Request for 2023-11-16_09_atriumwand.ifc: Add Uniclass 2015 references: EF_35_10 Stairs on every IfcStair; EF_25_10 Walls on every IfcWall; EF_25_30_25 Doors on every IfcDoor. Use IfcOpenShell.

First a look at what the model holds.

```python
import ifcopenshell

model = ifcopenshell.open("2023-11-16_09_atriumwand.ifc")
print(model.schema)
print("classifications:", [c.Name for c in model.by_type("IfcClassification")])
for ifc_class in ("IfcDoor", "IfcRoof", "IfcStair", "IfcWall", "IfcWindow"):
    print(ifc_class, len(model.by_type(ifc_class)))
```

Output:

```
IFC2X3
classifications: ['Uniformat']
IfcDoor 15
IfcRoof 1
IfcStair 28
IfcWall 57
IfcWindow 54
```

```python
import ifcopenshell
import ifcopenshell.api.classification

model = ifcopenshell.open("2023-11-16_09_atriumwand.ifc")

# IFC2X3 requires Source and Edition and has no link from the project to the system.
system = model.create_entity("IfcClassification", Source="NBS", Edition="2015", Name="Uniclass 2015")

codes = {
    "IfcStair": ("EF_35_10", "Stairs"),
    "IfcWall": ("EF_25_10", "Walls"),
    "IfcDoor": ("EF_25_30_25", "Doors"),
}
for ifc_class, (code, name) in codes.items():
    products = model.by_type(ifc_class)
    ifcopenshell.api.classification.add_reference(
        model, products=products, classification=system, identification=code, name=name
    )
    print(code, len(products))

model.write("2023-11-16_09_atriumwand_edited.ifc")
```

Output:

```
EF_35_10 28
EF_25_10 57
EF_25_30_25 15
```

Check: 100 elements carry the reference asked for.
